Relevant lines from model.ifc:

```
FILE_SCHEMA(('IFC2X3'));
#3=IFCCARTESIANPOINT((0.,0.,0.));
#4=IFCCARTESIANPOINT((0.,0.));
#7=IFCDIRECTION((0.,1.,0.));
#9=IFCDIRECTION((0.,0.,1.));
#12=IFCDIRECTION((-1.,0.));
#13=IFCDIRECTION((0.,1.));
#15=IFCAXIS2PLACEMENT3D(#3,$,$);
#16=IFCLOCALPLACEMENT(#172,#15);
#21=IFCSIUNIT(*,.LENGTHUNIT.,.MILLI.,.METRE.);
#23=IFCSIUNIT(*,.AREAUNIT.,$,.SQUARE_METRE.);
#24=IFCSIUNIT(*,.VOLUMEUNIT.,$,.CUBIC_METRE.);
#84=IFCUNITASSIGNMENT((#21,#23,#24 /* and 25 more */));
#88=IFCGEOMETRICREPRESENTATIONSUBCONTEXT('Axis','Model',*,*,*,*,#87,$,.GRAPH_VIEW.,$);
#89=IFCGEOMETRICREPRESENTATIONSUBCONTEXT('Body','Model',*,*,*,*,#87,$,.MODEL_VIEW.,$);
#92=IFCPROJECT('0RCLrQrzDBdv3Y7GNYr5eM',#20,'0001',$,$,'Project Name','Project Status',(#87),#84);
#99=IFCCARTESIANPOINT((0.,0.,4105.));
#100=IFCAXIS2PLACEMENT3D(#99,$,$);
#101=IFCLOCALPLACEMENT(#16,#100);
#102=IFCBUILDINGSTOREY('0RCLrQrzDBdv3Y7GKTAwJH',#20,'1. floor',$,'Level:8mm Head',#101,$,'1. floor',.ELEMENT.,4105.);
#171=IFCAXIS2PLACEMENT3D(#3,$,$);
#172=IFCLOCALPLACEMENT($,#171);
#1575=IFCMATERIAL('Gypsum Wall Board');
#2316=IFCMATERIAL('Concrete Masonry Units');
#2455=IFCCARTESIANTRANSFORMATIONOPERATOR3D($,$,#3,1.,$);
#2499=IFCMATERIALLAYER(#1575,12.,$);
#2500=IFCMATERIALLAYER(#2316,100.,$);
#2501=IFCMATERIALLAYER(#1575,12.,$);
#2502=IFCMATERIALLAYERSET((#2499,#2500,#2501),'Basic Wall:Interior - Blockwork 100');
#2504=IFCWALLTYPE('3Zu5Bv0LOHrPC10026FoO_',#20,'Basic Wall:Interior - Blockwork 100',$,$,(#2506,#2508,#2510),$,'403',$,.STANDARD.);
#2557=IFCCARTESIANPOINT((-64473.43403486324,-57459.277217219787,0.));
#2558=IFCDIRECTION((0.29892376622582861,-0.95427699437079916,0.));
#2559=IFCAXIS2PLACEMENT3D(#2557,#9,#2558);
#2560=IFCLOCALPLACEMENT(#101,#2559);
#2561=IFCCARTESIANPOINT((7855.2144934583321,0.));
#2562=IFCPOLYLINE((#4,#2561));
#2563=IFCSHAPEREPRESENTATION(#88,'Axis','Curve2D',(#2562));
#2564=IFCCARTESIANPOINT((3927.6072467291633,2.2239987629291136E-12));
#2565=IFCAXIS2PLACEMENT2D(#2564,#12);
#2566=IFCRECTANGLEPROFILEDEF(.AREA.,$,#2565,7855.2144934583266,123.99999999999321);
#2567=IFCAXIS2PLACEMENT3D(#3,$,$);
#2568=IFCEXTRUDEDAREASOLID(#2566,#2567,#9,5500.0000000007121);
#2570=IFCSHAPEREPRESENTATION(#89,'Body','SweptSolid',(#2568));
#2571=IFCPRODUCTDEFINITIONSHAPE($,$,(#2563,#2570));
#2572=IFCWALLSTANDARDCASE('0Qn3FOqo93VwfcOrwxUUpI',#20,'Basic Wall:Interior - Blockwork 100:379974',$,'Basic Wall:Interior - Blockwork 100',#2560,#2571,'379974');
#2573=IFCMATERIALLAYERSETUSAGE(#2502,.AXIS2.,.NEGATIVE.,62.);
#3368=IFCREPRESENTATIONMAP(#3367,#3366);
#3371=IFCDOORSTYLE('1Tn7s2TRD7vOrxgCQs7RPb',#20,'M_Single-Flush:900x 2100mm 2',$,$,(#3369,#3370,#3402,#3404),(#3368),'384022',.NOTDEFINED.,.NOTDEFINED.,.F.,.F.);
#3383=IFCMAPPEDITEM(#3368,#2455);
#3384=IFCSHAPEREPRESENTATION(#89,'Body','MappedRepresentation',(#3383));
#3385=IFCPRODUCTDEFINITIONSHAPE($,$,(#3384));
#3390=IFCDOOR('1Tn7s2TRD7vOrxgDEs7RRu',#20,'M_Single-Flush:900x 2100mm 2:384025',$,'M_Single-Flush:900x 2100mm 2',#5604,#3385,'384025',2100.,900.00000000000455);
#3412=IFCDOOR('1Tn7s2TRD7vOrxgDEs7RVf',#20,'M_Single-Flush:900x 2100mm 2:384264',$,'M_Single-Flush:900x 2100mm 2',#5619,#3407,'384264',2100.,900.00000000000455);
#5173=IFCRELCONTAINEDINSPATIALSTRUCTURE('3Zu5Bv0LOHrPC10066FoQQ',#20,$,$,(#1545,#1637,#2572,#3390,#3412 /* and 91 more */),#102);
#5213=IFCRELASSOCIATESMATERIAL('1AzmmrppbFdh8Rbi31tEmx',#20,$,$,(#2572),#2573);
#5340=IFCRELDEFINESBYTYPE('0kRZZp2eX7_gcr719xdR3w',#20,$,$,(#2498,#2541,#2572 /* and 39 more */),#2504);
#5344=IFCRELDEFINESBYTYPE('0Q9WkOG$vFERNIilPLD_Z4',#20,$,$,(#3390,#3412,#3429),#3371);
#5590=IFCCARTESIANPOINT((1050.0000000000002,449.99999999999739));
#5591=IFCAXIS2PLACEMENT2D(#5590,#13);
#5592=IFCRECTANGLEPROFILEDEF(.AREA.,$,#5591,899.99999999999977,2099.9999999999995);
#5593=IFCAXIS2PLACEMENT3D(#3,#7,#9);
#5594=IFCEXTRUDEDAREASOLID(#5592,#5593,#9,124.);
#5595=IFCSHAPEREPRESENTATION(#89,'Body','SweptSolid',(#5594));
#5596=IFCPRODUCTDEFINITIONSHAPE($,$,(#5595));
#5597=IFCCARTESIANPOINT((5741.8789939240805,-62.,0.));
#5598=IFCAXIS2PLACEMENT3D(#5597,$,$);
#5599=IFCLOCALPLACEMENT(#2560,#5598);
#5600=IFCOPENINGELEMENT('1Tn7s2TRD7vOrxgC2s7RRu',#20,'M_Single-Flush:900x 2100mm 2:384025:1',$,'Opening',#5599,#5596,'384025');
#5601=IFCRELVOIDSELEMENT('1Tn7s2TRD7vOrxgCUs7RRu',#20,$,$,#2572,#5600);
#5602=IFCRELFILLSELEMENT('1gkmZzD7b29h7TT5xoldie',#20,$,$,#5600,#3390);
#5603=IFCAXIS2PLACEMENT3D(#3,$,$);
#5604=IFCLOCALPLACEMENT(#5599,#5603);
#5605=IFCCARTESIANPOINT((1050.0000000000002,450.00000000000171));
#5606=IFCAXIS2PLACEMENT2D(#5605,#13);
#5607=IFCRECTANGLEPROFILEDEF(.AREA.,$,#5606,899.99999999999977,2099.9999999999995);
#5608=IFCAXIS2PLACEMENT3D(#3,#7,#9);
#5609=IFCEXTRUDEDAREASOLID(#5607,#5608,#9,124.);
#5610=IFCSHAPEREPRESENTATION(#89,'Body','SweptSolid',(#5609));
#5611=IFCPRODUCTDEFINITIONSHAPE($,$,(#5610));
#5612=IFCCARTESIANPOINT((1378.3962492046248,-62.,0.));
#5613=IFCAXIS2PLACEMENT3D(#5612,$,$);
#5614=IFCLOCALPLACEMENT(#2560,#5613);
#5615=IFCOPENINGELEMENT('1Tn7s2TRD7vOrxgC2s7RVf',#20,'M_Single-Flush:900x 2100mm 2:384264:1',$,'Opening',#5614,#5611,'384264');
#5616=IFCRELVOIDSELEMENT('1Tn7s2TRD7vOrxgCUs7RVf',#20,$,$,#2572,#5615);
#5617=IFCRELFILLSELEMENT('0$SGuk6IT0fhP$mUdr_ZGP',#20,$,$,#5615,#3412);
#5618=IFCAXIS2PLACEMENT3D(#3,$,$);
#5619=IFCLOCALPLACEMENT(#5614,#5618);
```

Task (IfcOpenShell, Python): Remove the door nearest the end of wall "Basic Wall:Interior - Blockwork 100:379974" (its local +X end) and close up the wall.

```python
import ifcopenshell
import ifcopenshell.api.feature
import ifcopenshell.api.root
import ifcopenshell.geom
import ifcopenshell.util.shape

model = ifcopenshell.open("model.ifc")
settings = ifcopenshell.geom.settings()


def volume(element):
    """Net volume in cubic metres, openings subtracted."""
    shape = ifcopenshell.geom.create_shape(settings, element)
    return ifcopenshell.util.shape.get_volume(shape.geometry)


door = model.by_id(3390)
opening = door.FillsVoids[0].RelatingOpeningElement
wall = opening.VoidsElements[0].RelatingBuildingElement
before = volume(wall)

ifcopenshell.api.root.remove_product(model, product=door)
ifcopenshell.api.feature.remove_feature(model, feature=opening)

after = volume(wall)

print(f"wall volume {before:.3f} -> {after:.3f} m3")

model.write("model_rev.ifc")
```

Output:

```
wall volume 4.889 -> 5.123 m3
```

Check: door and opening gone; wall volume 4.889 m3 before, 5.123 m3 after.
